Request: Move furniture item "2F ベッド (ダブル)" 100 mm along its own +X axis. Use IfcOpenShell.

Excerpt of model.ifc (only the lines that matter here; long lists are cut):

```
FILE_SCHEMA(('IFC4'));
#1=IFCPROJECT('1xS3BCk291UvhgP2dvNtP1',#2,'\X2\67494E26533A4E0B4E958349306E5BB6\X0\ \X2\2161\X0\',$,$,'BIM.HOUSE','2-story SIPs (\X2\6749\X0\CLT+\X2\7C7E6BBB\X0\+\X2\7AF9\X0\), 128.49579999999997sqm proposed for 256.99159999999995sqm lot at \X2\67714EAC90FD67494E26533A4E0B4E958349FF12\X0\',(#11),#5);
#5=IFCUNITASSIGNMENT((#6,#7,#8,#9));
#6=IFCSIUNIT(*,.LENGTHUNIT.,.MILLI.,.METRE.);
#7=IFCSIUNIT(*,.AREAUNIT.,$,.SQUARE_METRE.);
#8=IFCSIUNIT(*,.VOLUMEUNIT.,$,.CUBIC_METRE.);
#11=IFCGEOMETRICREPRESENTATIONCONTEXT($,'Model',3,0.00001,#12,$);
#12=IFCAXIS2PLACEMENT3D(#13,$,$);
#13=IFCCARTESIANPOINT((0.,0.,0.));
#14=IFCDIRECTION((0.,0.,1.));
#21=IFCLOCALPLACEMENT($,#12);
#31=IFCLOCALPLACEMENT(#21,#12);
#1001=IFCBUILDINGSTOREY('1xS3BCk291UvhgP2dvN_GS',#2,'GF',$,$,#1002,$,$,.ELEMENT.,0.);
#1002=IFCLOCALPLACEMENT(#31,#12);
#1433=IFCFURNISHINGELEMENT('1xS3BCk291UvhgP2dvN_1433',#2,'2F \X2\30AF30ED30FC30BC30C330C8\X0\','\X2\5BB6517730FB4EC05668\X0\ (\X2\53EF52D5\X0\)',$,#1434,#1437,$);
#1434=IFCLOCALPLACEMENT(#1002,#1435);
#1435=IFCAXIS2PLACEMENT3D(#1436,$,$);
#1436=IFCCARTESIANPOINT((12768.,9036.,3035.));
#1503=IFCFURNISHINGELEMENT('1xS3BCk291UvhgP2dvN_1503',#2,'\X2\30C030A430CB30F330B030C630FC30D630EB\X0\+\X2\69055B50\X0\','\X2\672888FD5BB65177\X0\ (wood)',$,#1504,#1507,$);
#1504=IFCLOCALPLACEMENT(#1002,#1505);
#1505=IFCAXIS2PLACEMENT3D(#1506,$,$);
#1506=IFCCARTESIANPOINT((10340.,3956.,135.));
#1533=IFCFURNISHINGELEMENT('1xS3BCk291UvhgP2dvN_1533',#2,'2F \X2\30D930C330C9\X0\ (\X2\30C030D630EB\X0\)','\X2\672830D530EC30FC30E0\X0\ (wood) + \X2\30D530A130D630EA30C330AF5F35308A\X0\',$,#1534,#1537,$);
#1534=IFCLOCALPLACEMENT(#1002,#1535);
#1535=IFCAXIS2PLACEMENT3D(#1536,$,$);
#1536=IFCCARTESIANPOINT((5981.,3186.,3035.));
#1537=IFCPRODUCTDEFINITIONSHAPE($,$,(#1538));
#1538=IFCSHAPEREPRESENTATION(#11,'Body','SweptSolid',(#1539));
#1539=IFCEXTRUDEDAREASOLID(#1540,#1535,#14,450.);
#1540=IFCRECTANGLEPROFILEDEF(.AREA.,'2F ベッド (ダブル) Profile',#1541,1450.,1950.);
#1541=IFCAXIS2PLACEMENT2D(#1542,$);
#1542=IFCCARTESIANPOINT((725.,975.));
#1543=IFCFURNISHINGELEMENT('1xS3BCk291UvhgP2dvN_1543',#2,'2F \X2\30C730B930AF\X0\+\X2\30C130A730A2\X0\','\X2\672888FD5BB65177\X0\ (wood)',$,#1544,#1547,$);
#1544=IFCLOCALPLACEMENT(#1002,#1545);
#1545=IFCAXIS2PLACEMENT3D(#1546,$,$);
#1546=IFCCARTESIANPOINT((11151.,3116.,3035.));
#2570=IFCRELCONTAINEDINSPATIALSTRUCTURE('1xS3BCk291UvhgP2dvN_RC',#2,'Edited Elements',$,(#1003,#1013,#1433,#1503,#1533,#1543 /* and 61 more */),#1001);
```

```python
import ifcopenshell
import ifcopenshell.api.geometry
import ifcopenshell.util.placement
import ifcopenshell.util.unit

model = ifcopenshell.open("model.ifc")
unit_scale = ifcopenshell.util.unit.calculate_unit_scale(model)

item = model.by_guid("1xS3BCk291UvhgP2dvN_1533")
matrix = ifcopenshell.util.placement.get_local_placement(item.ObjectPlacement)
matrix[:3, 3] += matrix[:3, 0] * 0.1 / unit_scale
ifcopenshell.api.geometry.edit_object_placement(model, product=item, matrix=matrix, is_si=False)

print(ifcopenshell.util.placement.get_local_placement(item.ObjectPlacement).round(3) + 0.0)

model.write("model_updated.ifc")
```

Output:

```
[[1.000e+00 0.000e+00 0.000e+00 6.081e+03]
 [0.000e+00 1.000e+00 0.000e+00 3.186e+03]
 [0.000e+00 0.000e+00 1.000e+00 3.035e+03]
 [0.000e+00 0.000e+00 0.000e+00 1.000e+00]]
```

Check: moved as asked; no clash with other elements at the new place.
